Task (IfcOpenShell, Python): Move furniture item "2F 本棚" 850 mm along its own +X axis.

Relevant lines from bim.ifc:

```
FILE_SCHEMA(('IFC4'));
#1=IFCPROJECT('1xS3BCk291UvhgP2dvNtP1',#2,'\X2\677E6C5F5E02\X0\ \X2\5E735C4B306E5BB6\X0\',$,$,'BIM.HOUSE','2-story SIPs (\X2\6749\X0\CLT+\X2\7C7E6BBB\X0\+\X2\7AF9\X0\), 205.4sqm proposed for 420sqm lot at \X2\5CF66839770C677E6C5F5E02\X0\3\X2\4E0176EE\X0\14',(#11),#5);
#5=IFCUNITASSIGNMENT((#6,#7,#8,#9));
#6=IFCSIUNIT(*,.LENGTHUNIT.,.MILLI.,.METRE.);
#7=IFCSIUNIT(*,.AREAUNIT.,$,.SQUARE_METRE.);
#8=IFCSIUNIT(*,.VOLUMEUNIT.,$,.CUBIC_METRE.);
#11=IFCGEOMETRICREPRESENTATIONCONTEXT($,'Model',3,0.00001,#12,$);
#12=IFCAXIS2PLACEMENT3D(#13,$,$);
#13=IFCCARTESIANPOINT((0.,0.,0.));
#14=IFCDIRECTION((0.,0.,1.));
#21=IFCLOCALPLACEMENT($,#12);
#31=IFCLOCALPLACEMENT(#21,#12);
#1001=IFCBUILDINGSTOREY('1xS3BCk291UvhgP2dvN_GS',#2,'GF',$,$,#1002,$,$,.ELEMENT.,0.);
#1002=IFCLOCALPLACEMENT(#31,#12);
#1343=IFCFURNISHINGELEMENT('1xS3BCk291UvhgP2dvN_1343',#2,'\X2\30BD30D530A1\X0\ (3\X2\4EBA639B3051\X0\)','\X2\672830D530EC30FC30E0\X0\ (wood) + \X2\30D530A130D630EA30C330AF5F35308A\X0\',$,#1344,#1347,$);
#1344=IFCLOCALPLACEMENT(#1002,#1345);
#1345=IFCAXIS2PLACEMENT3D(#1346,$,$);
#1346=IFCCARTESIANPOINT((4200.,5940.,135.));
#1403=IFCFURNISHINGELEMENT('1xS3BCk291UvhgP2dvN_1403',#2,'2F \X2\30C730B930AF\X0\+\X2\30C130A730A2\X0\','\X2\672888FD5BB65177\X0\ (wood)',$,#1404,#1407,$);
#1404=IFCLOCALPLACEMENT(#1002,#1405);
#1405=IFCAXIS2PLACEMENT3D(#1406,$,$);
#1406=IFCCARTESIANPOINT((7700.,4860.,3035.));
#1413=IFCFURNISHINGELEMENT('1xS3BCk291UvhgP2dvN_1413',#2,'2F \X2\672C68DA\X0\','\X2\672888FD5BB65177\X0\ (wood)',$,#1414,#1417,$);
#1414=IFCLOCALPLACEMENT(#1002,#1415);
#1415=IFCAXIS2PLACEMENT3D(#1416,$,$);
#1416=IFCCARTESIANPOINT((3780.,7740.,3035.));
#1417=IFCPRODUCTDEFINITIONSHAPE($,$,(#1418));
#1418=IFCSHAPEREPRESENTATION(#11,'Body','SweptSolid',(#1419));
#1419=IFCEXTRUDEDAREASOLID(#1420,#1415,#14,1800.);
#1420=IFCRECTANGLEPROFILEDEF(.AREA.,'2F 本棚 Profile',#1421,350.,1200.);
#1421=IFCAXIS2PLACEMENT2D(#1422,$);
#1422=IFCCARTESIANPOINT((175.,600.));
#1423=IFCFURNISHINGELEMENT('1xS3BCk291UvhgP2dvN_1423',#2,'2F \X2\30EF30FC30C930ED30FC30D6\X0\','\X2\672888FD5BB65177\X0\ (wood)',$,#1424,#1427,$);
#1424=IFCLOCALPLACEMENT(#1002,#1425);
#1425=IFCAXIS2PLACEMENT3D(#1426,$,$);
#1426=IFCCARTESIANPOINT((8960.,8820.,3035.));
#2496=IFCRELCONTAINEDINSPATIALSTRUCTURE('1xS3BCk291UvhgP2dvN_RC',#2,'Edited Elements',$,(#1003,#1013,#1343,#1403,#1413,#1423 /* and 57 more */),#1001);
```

```python
import ifcopenshell
import ifcopenshell.api.geometry
import ifcopenshell.util.placement

model = ifcopenshell.open("bim.ifc")

item = model.by_guid("1xS3BCk291UvhgP2dvN_1413")
matrix = ifcopenshell.util.placement.get_local_placement(item.ObjectPlacement)
matrix[:3, 3] += matrix[:3, 0] * 850.0
ifcopenshell.api.geometry.edit_object_placement(model, product=item, matrix=matrix, is_si=False)

print(ifcopenshell.util.placement.get_local_placement(item.ObjectPlacement).round(3) + 0.0)

model.write("bim_updated.ifc")
```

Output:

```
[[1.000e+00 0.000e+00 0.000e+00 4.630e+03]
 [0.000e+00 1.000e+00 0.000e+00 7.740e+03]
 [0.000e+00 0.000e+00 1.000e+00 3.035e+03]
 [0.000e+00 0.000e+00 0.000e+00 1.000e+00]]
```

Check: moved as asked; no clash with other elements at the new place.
